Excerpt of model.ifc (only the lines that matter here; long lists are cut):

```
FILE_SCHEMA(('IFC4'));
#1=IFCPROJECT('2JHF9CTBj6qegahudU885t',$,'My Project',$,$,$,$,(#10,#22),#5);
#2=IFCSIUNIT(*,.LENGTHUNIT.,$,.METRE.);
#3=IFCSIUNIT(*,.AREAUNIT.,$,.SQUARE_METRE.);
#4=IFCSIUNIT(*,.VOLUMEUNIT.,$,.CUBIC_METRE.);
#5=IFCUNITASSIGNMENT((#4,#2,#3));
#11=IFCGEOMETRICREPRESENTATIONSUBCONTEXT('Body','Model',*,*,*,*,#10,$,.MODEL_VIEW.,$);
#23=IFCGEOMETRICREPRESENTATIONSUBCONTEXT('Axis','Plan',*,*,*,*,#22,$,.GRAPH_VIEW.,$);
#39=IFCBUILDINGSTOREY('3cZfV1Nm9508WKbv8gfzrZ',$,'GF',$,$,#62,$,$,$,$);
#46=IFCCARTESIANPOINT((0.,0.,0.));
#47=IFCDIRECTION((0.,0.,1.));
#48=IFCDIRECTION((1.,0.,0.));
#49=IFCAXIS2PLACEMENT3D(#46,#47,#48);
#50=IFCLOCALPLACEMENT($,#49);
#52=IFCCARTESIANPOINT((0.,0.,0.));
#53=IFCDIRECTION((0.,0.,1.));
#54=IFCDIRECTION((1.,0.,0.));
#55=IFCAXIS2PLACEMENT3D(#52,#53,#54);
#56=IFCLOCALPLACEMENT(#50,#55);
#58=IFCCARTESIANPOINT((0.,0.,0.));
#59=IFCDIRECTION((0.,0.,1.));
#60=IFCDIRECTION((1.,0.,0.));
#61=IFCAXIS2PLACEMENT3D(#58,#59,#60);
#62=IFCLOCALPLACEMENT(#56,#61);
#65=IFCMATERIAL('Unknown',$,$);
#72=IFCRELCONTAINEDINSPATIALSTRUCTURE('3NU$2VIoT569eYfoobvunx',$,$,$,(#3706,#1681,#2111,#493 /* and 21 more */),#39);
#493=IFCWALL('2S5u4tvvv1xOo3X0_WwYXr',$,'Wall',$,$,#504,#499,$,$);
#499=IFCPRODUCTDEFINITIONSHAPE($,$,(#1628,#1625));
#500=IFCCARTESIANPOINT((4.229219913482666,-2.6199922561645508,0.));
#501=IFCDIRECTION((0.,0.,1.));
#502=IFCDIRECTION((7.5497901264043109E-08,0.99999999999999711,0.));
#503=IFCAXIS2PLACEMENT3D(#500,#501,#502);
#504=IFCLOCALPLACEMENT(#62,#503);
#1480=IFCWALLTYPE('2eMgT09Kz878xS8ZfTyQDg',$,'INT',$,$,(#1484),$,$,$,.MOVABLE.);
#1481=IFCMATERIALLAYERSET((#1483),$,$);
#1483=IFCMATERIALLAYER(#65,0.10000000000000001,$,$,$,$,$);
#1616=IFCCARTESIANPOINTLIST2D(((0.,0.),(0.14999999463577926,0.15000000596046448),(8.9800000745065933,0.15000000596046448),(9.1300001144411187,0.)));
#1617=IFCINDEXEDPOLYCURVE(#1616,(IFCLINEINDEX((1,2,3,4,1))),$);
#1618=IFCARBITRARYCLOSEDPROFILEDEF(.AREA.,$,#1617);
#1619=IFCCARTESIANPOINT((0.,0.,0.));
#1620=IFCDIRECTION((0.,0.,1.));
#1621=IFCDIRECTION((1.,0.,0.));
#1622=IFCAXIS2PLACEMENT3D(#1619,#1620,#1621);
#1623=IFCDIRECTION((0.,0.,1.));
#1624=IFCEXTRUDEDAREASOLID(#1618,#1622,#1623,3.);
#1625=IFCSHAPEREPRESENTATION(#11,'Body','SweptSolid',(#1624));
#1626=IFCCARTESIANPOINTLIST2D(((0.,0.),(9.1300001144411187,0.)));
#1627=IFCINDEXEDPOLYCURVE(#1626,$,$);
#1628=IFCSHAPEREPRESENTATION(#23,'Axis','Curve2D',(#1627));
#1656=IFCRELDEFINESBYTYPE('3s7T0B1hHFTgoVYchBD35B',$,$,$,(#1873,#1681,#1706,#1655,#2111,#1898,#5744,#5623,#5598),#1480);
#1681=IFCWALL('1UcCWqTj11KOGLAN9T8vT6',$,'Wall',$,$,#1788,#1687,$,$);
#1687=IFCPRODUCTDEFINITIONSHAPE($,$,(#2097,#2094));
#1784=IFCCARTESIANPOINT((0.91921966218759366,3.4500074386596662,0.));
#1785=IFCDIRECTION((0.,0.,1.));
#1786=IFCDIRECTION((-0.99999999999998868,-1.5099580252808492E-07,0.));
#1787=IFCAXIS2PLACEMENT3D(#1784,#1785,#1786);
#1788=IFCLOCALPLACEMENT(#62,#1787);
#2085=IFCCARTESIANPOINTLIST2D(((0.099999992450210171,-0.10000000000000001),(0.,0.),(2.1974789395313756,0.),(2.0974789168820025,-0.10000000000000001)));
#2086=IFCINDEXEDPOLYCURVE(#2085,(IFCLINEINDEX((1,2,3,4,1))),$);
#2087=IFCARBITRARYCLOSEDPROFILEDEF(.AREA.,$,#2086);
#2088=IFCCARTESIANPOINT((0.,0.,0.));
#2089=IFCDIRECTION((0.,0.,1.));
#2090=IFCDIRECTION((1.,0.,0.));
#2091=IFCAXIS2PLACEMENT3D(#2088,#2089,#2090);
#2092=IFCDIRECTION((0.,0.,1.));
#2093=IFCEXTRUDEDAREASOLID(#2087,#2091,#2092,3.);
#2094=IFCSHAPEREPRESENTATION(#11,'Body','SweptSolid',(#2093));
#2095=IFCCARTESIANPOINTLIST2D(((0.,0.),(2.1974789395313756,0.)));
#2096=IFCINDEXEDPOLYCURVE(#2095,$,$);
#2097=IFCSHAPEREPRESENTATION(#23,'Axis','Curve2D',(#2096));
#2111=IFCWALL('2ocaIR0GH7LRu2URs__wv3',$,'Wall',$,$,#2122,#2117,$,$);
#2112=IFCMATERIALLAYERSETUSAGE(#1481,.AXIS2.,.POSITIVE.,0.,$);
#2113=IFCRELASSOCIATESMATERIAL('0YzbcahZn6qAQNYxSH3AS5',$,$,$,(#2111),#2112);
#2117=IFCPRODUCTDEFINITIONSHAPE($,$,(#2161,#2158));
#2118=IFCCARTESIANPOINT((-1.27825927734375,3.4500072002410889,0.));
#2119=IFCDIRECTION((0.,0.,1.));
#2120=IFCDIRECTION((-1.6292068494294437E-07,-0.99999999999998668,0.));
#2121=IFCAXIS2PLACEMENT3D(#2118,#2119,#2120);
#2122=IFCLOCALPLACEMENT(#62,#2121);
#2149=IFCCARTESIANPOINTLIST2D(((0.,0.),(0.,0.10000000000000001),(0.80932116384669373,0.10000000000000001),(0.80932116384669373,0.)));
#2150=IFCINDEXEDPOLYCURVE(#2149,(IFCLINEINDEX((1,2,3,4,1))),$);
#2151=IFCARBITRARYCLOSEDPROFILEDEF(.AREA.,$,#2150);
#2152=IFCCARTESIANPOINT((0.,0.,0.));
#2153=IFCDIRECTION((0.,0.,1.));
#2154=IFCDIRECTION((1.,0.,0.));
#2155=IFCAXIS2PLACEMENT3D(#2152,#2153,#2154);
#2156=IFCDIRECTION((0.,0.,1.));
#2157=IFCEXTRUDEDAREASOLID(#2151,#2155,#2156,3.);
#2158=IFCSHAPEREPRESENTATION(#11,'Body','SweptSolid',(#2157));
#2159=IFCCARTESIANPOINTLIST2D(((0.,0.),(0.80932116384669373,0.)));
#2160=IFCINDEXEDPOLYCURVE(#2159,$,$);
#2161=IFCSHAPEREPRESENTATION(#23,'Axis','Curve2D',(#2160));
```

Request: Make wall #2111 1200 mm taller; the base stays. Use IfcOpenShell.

```python
import ifcopenshell
import ifcopenshell.geom
import ifcopenshell.util.representation
import ifcopenshell.util.shape

model = ifcopenshell.open("model.ifc")
settings = ifcopenshell.geom.settings()


def volume(element):
    """Net volume in cubic metres, openings subtracted."""
    shape = ifcopenshell.geom.create_shape(settings, element)
    return ifcopenshell.util.shape.get_volume(shape.geometry)


wall = model.by_guid("2ocaIR0GH7LRu2URs__wv3")
before = volume(wall)

body = ifcopenshell.util.representation.get_representation(wall, "Model", "Body")
solid = body.Items[0]
old_height = solid.Depth
solid.Depth += 1.2
after = volume(wall)

print(f"height {old_height:g} -> {solid.Depth:g}, volume {before:.3f} -> {after:.3f} m3")

model.write("model_rev.ifc")
```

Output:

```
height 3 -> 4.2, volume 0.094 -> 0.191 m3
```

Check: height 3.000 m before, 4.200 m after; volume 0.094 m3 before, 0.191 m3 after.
